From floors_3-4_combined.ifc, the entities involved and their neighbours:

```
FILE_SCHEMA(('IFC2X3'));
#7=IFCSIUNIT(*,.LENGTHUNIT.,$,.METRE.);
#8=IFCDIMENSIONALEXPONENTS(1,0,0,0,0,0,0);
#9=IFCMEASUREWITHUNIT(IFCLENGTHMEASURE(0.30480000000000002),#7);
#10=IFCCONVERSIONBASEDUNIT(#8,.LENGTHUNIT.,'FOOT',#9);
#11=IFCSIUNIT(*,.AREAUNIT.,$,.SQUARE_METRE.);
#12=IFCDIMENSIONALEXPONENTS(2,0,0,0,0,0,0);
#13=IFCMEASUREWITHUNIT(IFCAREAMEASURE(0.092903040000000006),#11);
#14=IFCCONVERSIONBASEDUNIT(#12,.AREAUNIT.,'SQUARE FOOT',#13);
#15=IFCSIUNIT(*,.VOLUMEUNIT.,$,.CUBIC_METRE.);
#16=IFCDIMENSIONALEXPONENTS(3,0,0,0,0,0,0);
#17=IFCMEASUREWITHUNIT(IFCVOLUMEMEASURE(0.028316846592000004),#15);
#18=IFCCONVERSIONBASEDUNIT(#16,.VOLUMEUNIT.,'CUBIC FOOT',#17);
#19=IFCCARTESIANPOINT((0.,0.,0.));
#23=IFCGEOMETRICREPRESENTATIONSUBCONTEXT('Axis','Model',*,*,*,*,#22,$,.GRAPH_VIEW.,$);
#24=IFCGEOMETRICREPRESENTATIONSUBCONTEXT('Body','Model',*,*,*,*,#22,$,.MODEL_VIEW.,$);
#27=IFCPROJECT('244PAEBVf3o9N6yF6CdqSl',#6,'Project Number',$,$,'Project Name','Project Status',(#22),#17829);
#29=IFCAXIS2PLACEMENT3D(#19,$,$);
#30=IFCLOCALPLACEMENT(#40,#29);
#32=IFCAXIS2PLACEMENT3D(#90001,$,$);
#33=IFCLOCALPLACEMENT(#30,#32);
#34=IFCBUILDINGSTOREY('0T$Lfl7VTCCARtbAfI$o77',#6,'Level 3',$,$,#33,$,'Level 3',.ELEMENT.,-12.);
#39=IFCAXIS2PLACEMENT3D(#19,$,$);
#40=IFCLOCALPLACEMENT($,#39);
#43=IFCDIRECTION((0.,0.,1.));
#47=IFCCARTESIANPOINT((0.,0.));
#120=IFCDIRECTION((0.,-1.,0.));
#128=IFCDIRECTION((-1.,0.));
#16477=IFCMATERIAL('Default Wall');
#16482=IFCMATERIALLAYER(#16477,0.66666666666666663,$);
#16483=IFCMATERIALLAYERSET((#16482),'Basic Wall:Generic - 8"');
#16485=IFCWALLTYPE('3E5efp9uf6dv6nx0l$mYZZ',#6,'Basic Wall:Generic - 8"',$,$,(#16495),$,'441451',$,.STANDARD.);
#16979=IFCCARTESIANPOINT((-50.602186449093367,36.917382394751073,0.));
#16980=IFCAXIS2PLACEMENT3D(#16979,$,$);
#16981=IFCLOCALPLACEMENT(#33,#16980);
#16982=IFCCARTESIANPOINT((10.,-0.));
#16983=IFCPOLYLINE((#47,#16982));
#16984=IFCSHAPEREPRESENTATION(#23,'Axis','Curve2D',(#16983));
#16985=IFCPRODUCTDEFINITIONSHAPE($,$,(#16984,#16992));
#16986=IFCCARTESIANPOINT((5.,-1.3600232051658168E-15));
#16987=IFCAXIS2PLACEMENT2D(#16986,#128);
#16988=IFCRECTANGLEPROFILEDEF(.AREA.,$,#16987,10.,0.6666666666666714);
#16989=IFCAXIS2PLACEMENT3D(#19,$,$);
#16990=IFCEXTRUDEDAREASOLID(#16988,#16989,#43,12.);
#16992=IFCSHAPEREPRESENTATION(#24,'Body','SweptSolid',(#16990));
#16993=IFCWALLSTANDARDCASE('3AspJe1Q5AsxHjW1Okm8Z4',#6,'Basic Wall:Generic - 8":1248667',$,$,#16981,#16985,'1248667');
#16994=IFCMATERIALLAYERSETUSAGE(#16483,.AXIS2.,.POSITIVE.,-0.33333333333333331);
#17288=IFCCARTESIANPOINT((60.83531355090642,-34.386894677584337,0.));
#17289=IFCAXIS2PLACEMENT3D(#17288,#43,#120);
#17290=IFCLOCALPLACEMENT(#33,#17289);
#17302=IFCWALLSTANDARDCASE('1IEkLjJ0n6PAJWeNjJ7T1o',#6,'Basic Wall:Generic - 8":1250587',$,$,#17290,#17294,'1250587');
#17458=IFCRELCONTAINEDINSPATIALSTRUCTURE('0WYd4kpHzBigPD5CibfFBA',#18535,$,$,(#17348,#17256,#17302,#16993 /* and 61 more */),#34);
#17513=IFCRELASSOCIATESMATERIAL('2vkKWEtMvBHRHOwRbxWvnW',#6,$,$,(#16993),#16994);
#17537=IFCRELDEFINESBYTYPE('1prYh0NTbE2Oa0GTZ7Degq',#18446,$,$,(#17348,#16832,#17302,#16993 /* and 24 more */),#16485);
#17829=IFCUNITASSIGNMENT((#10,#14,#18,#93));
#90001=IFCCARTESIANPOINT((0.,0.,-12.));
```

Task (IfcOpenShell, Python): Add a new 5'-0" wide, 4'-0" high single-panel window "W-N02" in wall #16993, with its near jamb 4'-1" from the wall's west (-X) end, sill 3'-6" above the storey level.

```python
import numpy as np
import ifcopenshell
import ifcopenshell.api.feature
import ifcopenshell.api.geometry
import ifcopenshell.api.root
import ifcopenshell.api.spatial
import ifcopenshell.api.type
import ifcopenshell.geom
import ifcopenshell.util.element
import ifcopenshell.util.placement
import ifcopenshell.util.representation
import ifcopenshell.util.shape
import ifcopenshell.util.unit

model = ifcopenshell.open("floors_3-4_combined.ifc")
unit_scale = ifcopenshell.util.unit.calculate_unit_scale(model)
settings = ifcopenshell.geom.settings()


def volume(element):
    """Net volume in cubic metres, openings subtracted."""
    shape = ifcopenshell.geom.create_shape(settings, element)
    return ifcopenshell.util.shape.get_volume(shape.geometry)


wall = model.by_guid("3AspJe1Q5AsxHjW1Okm8Z4")
storey = ifcopenshell.util.element.get_container(wall, ifc_class="IfcBuildingStorey")
context = ifcopenshell.util.representation.get_context(model, "Model", "Body", "MODEL_VIEW")
before = volume(wall)

width, height, from_end, sill = 1.524, 1.2192, 1.2446, 1.0668  # metres

# The wall runs along its own X axis, and the end named is its -X end.
wall_shape = ifcopenshell.geom.create_shape(settings, wall)
x, y, z = ifcopenshell.util.shape.get_vertices(wall_shape.geometry).T
start = x.min() + from_end
face, thickness = float(y.min()), float(y.max() - y.min())
wall_matrix = ifcopenshell.util.placement.get_local_placement(wall.ObjectPlacement)
level = ifcopenshell.util.placement.get_local_placement(storey.ObjectPlacement)[2, 3]


def in_wall(x, y):
    """Placement at x, y metres in the wall's axes, at sill height."""
    matrix = wall_matrix.copy()
    matrix[:, 3] = wall_matrix @ np.array([x / unit_scale, y / unit_scale, 0.0, 1.0])
    matrix[2, 3] = level + sill / unit_scale
    return matrix


# Opening: a box that overshoots both wall faces by 50 mm.
opening = ifcopenshell.api.root.create_entity(model, ifc_class="IfcOpeningElement")
box = ifcopenshell.api.geometry.add_wall_representation(
    model, context=context, length=width, height=height, thickness=thickness + 0.1
)
ifcopenshell.api.geometry.assign_representation(model, product=opening, representation=box)
ifcopenshell.api.geometry.edit_object_placement(model, product=opening, matrix=in_wall(start, face - 0.05), is_si=False)
ifcopenshell.api.feature.add_feature(model, feature=opening, element=wall)

window = ifcopenshell.api.root.create_entity(model, ifc_class="IfcWindow", name="W-N02")
window.OverallWidth, window.OverallHeight = width / unit_scale, height / unit_scale
body = ifcopenshell.api.geometry.add_window_representation(
    model,
    context=context,
    overall_width=window.OverallWidth,
    overall_height=window.OverallHeight,
    partition_type="SINGLE_PANEL",
)
ifcopenshell.api.geometry.assign_representation(model, product=window, representation=body)
ifcopenshell.api.spatial.assign_container(model, products=[window], relating_structure=storey)
fills = ifcopenshell.api.feature.add_filling(model, opening=opening, element=window)
fills.OwnerHistory = window.OwnerHistory  # required in IFC2X3

# IFC2X3 keeps the operation on the window style.
style = ifcopenshell.api.root.create_entity(model, ifc_class="IfcWindowStyle", name="W-N02")
style.OperationType, style.ConstructionType = "SINGLE_PANEL", "NOTDEFINED"
style.ParameterTakesPrecedence = style.Sizeable = False
ifcopenshell.api.type.assign_type(model, related_objects=[window], relating_type=style)

# Centre the window in the wall's thickness.
ifcopenshell.api.geometry.edit_object_placement(model, product=window, matrix=in_wall(start, face), is_si=False)
window_shape = ifcopenshell.geom.create_shape(settings, window)
depth = ifcopenshell.util.shape.get_vertices(window_shape.geometry)[:, 1]
offset = face + thickness / 2 - (depth.min() + depth.max()) / 2
ifcopenshell.api.geometry.edit_object_placement(model, product=window, matrix=in_wall(start, offset), is_si=False)

after = volume(wall)

print(f"wall volume {before:.3f} -> {after:.3f} m3")

model.write("floors_3-4_combined_edited.ifc")
```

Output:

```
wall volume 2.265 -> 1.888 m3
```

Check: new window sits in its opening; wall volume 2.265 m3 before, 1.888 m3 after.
